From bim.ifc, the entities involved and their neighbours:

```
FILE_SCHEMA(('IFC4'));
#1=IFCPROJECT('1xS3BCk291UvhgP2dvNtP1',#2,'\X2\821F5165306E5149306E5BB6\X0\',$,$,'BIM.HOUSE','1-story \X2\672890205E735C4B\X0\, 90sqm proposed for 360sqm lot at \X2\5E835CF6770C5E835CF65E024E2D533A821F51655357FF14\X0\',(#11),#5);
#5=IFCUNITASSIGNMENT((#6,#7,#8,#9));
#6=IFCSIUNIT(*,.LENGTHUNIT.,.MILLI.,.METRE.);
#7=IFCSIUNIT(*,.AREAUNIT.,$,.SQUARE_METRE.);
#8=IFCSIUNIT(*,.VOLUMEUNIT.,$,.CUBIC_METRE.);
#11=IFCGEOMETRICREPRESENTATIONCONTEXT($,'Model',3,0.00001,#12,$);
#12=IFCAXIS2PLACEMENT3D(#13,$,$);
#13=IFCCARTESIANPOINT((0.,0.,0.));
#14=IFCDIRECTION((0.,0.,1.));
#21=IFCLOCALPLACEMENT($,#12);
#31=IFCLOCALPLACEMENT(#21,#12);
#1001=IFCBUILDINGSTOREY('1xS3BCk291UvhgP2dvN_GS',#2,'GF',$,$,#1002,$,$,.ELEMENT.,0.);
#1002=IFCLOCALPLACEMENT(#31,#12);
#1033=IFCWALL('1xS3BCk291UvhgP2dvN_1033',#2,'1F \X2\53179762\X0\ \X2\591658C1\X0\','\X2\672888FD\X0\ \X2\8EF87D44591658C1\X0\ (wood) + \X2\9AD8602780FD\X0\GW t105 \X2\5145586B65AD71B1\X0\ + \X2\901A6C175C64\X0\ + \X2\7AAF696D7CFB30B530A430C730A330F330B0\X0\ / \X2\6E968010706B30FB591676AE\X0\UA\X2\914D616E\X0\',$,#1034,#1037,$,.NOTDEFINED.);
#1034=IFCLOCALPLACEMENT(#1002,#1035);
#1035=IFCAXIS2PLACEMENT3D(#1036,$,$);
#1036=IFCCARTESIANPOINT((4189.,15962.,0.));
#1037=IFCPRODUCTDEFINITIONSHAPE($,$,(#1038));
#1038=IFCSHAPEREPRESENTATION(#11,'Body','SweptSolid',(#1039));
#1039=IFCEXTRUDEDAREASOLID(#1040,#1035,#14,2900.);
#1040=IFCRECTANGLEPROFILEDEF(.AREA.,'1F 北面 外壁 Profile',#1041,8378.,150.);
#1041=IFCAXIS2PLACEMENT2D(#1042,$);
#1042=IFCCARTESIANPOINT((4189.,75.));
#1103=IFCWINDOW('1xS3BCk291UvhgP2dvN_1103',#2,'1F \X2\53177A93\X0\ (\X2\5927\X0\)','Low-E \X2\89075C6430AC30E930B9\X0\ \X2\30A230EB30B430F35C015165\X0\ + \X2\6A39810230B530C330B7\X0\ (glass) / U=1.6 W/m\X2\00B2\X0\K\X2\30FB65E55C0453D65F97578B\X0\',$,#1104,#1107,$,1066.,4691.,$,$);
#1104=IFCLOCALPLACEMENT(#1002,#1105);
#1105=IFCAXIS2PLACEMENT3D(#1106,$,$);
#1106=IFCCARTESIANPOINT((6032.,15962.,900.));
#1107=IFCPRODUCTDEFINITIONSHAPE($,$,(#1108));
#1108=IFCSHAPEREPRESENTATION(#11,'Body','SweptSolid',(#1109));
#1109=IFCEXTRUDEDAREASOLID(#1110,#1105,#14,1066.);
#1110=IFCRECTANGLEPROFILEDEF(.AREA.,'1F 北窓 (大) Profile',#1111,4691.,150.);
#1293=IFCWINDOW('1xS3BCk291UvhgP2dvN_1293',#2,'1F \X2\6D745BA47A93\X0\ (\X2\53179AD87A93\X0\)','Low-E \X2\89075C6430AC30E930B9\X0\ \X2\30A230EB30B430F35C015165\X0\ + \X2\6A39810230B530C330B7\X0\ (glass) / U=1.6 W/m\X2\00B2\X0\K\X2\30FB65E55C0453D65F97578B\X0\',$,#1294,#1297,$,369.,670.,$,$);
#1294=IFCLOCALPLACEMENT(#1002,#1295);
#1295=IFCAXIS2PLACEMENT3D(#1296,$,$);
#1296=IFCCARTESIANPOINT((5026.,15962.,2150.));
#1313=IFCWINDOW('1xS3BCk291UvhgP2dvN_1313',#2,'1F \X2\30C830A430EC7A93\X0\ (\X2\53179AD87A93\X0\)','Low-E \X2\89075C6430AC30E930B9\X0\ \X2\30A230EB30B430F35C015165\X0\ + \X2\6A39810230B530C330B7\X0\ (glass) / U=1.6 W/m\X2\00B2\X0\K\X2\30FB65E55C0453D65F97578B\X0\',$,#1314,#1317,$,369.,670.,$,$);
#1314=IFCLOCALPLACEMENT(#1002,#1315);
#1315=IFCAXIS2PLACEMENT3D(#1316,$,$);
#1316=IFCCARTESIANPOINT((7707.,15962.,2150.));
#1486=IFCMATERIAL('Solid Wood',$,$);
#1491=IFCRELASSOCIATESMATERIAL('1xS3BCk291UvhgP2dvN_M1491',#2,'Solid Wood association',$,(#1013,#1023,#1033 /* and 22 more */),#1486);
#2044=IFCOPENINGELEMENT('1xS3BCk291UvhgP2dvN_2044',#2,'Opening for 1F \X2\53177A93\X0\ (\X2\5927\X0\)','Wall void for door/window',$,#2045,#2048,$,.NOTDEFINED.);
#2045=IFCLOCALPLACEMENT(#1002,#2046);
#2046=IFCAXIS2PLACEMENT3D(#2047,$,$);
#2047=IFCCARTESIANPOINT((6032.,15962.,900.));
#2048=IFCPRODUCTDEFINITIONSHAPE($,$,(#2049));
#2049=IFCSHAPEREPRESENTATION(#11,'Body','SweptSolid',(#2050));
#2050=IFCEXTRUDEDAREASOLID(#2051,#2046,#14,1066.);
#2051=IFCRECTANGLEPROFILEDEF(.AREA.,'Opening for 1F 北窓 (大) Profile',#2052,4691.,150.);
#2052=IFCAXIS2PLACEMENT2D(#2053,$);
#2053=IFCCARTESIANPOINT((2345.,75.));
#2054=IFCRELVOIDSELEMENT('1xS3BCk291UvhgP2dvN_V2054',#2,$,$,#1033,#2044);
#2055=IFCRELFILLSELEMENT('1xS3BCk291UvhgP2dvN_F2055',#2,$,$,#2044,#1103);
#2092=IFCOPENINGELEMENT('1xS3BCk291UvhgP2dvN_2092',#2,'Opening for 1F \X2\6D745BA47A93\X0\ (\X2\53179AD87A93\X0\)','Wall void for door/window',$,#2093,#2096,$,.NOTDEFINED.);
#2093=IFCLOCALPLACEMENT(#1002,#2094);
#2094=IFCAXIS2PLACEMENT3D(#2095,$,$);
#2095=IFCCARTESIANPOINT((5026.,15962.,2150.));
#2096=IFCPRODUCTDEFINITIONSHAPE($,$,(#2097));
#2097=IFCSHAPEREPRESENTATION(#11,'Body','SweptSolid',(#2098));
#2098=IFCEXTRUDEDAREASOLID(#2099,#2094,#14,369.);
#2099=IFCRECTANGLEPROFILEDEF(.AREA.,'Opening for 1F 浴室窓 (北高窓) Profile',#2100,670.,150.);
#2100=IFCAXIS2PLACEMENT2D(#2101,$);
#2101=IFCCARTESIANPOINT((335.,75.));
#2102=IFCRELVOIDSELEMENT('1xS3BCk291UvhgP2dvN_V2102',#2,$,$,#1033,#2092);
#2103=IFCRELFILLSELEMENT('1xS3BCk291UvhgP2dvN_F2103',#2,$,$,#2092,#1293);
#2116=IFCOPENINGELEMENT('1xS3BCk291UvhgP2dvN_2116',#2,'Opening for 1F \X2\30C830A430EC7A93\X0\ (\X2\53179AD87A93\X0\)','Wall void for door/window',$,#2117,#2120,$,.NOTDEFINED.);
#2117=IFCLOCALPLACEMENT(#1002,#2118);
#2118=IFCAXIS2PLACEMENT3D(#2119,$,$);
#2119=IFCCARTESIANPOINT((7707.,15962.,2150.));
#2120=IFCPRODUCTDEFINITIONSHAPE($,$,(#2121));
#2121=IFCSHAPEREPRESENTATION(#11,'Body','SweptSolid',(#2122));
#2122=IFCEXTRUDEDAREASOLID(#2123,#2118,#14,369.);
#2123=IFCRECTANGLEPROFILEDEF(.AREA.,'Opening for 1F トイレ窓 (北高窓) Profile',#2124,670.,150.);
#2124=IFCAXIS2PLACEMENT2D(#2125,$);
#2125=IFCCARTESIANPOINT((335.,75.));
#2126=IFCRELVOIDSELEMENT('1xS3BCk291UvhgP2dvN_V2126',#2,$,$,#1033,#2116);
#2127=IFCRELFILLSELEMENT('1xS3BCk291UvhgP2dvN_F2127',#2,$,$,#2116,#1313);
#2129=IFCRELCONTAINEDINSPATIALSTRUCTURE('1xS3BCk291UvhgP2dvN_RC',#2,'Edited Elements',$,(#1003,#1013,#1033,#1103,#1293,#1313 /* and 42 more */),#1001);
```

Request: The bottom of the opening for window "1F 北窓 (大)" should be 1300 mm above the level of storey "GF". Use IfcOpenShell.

```python
import numpy as np
import ifcopenshell
import ifcopenshell.api.geometry
import ifcopenshell.geom
import ifcopenshell.util.element
import ifcopenshell.util.placement
import ifcopenshell.util.shape
import ifcopenshell.util.unit

model = ifcopenshell.open("bim.ifc")
unit_scale = ifcopenshell.util.unit.calculate_unit_scale(model)

window = model.by_guid("1xS3BCk291UvhgP2dvN_1103")
opening = window.FillsVoids[0].RelatingOpeningElement
storey = ifcopenshell.util.element.get_container(window, ifc_class="IfcBuildingStorey")
level = ifcopenshell.util.placement.get_local_placement(storey.ObjectPlacement)[2, 3]

# The opening's origin need not be at the sill, so measure its lowest point.
shape = ifcopenshell.geom.create_shape(ifcopenshell.geom.settings(), opening)
bottom = ifcopenshell.util.shape.get_shape_bottom_elevation(shape, shape.geometry) / unit_scale
dz = level + 1.3 / unit_scale - bottom

shift = np.array([0.0, 0.0, dz])
# The window is not placed relative to its opening, so move both.
for product in (opening, window):
    matrix = ifcopenshell.util.placement.get_local_placement(product.ObjectPlacement)
    matrix[:3, 3] += shift
    ifcopenshell.api.geometry.edit_object_placement(model, product=product, matrix=matrix, is_si=False)

print(f"moved by {dz * unit_scale:+.3f} m")

model.write("bim-out.ifc")
```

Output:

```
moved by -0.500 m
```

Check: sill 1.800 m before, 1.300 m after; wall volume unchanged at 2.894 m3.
